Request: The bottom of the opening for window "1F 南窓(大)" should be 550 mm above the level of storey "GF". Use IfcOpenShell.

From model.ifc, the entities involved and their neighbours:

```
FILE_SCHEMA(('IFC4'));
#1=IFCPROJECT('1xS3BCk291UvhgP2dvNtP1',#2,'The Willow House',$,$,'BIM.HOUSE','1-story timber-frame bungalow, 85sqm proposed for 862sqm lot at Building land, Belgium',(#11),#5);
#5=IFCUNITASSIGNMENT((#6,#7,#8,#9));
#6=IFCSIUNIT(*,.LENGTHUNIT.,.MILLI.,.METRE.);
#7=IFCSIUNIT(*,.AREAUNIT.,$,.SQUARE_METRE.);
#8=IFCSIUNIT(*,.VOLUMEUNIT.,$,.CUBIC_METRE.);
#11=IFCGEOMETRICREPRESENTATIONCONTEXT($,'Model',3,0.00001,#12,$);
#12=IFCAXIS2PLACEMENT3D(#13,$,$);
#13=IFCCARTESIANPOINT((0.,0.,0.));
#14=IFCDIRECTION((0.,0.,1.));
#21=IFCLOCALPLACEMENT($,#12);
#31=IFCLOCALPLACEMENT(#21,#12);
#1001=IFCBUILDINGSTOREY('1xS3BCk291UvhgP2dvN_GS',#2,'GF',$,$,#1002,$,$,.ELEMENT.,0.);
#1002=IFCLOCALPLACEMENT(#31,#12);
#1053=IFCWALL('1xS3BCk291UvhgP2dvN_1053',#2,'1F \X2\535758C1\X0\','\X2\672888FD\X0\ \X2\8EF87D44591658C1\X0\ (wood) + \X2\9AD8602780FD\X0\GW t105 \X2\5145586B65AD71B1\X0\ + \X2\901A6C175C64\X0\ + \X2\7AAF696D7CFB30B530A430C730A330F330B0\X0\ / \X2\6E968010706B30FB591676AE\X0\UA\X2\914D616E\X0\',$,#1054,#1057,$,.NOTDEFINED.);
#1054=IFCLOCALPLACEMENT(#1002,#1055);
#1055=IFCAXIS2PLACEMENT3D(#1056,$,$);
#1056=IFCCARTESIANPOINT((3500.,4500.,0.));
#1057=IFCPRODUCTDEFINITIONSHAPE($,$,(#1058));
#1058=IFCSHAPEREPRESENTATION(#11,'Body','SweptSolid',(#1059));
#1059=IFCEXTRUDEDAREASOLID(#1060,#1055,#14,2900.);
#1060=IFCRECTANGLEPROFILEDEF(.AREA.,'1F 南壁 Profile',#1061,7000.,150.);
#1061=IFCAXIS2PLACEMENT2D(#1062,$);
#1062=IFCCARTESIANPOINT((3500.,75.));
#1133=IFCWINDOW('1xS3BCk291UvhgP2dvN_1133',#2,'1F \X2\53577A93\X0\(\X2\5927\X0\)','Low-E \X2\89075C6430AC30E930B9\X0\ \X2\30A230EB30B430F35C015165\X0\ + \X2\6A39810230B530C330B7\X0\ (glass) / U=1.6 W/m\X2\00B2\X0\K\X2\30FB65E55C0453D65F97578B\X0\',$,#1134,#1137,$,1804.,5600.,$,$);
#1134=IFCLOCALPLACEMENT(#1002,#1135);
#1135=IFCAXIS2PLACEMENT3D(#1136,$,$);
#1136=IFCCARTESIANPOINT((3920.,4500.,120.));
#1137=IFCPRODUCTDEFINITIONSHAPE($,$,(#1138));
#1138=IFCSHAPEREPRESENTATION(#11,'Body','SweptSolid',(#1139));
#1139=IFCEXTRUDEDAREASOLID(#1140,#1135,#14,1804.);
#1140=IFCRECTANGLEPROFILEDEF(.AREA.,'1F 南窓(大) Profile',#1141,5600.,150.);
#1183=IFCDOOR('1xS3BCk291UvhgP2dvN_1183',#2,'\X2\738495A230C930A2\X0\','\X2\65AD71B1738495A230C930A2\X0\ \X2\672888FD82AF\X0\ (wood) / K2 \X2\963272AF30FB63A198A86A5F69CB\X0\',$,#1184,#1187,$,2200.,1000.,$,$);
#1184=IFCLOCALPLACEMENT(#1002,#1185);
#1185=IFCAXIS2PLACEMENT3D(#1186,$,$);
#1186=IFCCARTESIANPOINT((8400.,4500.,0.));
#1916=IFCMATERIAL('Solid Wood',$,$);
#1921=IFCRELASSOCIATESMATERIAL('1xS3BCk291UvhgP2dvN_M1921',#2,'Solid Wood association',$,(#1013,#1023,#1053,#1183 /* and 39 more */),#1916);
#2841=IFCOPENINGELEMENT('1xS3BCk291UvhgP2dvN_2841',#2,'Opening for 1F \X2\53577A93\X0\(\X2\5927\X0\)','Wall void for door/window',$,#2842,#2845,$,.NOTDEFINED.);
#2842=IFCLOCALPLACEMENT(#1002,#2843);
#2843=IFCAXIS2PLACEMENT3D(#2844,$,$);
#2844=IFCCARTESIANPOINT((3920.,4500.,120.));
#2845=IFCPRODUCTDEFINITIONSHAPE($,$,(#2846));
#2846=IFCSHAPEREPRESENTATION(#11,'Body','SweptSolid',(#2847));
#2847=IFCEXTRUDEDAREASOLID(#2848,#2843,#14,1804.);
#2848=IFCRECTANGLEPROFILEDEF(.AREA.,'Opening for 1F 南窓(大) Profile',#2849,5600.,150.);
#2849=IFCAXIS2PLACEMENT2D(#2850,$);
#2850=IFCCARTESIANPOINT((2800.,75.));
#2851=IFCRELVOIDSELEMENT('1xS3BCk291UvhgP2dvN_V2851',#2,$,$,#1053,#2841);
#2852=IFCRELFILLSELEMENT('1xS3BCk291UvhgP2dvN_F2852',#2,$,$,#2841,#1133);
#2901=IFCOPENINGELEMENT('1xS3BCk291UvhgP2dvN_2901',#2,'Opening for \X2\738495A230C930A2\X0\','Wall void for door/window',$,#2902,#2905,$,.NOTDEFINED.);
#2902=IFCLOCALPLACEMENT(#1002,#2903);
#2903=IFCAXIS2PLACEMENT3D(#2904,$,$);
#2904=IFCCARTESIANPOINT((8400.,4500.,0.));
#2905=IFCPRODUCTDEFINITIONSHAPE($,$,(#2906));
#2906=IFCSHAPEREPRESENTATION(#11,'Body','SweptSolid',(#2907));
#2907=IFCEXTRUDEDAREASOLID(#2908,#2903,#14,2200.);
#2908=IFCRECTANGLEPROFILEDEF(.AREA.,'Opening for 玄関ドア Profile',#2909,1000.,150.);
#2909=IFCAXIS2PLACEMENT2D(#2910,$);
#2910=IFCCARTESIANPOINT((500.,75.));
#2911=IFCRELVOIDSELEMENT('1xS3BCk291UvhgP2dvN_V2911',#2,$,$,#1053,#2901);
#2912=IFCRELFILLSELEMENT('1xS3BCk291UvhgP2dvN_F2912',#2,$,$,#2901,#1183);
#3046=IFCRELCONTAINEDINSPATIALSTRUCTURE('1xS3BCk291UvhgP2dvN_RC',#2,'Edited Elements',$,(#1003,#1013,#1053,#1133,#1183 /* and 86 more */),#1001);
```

```python
import numpy as np
import ifcopenshell
import ifcopenshell.api.geometry
import ifcopenshell.geom
import ifcopenshell.util.element
import ifcopenshell.util.placement
import ifcopenshell.util.shape
import ifcopenshell.util.unit

model = ifcopenshell.open("model.ifc")
unit_scale = ifcopenshell.util.unit.calculate_unit_scale(model)

window = model.by_guid("1xS3BCk291UvhgP2dvN_1133")
opening = window.FillsVoids[0].RelatingOpeningElement
storey = ifcopenshell.util.element.get_container(window, ifc_class="IfcBuildingStorey")
level = ifcopenshell.util.placement.get_local_placement(storey.ObjectPlacement)[2, 3]

# The opening's origin need not be at the sill, so measure its lowest point.
shape = ifcopenshell.geom.create_shape(ifcopenshell.geom.settings(), opening)
bottom = ifcopenshell.util.shape.get_shape_bottom_elevation(shape, shape.geometry) / unit_scale
dz = level + 550.0 - bottom

shift = np.array([0.0, 0.0, dz])
# The window is not placed relative to its opening, so move both.
for product in (opening, window):
    matrix = ifcopenshell.util.placement.get_local_placement(product.ObjectPlacement)
    matrix[:3, 3] += shift
    ifcopenshell.api.geometry.edit_object_placement(model, product=product, matrix=matrix, is_si=False)

print(f"moved by {dz * unit_scale:+.3f} m")

model.write("model_v2.ifc")
```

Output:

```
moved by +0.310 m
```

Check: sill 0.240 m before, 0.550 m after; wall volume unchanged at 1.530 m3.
